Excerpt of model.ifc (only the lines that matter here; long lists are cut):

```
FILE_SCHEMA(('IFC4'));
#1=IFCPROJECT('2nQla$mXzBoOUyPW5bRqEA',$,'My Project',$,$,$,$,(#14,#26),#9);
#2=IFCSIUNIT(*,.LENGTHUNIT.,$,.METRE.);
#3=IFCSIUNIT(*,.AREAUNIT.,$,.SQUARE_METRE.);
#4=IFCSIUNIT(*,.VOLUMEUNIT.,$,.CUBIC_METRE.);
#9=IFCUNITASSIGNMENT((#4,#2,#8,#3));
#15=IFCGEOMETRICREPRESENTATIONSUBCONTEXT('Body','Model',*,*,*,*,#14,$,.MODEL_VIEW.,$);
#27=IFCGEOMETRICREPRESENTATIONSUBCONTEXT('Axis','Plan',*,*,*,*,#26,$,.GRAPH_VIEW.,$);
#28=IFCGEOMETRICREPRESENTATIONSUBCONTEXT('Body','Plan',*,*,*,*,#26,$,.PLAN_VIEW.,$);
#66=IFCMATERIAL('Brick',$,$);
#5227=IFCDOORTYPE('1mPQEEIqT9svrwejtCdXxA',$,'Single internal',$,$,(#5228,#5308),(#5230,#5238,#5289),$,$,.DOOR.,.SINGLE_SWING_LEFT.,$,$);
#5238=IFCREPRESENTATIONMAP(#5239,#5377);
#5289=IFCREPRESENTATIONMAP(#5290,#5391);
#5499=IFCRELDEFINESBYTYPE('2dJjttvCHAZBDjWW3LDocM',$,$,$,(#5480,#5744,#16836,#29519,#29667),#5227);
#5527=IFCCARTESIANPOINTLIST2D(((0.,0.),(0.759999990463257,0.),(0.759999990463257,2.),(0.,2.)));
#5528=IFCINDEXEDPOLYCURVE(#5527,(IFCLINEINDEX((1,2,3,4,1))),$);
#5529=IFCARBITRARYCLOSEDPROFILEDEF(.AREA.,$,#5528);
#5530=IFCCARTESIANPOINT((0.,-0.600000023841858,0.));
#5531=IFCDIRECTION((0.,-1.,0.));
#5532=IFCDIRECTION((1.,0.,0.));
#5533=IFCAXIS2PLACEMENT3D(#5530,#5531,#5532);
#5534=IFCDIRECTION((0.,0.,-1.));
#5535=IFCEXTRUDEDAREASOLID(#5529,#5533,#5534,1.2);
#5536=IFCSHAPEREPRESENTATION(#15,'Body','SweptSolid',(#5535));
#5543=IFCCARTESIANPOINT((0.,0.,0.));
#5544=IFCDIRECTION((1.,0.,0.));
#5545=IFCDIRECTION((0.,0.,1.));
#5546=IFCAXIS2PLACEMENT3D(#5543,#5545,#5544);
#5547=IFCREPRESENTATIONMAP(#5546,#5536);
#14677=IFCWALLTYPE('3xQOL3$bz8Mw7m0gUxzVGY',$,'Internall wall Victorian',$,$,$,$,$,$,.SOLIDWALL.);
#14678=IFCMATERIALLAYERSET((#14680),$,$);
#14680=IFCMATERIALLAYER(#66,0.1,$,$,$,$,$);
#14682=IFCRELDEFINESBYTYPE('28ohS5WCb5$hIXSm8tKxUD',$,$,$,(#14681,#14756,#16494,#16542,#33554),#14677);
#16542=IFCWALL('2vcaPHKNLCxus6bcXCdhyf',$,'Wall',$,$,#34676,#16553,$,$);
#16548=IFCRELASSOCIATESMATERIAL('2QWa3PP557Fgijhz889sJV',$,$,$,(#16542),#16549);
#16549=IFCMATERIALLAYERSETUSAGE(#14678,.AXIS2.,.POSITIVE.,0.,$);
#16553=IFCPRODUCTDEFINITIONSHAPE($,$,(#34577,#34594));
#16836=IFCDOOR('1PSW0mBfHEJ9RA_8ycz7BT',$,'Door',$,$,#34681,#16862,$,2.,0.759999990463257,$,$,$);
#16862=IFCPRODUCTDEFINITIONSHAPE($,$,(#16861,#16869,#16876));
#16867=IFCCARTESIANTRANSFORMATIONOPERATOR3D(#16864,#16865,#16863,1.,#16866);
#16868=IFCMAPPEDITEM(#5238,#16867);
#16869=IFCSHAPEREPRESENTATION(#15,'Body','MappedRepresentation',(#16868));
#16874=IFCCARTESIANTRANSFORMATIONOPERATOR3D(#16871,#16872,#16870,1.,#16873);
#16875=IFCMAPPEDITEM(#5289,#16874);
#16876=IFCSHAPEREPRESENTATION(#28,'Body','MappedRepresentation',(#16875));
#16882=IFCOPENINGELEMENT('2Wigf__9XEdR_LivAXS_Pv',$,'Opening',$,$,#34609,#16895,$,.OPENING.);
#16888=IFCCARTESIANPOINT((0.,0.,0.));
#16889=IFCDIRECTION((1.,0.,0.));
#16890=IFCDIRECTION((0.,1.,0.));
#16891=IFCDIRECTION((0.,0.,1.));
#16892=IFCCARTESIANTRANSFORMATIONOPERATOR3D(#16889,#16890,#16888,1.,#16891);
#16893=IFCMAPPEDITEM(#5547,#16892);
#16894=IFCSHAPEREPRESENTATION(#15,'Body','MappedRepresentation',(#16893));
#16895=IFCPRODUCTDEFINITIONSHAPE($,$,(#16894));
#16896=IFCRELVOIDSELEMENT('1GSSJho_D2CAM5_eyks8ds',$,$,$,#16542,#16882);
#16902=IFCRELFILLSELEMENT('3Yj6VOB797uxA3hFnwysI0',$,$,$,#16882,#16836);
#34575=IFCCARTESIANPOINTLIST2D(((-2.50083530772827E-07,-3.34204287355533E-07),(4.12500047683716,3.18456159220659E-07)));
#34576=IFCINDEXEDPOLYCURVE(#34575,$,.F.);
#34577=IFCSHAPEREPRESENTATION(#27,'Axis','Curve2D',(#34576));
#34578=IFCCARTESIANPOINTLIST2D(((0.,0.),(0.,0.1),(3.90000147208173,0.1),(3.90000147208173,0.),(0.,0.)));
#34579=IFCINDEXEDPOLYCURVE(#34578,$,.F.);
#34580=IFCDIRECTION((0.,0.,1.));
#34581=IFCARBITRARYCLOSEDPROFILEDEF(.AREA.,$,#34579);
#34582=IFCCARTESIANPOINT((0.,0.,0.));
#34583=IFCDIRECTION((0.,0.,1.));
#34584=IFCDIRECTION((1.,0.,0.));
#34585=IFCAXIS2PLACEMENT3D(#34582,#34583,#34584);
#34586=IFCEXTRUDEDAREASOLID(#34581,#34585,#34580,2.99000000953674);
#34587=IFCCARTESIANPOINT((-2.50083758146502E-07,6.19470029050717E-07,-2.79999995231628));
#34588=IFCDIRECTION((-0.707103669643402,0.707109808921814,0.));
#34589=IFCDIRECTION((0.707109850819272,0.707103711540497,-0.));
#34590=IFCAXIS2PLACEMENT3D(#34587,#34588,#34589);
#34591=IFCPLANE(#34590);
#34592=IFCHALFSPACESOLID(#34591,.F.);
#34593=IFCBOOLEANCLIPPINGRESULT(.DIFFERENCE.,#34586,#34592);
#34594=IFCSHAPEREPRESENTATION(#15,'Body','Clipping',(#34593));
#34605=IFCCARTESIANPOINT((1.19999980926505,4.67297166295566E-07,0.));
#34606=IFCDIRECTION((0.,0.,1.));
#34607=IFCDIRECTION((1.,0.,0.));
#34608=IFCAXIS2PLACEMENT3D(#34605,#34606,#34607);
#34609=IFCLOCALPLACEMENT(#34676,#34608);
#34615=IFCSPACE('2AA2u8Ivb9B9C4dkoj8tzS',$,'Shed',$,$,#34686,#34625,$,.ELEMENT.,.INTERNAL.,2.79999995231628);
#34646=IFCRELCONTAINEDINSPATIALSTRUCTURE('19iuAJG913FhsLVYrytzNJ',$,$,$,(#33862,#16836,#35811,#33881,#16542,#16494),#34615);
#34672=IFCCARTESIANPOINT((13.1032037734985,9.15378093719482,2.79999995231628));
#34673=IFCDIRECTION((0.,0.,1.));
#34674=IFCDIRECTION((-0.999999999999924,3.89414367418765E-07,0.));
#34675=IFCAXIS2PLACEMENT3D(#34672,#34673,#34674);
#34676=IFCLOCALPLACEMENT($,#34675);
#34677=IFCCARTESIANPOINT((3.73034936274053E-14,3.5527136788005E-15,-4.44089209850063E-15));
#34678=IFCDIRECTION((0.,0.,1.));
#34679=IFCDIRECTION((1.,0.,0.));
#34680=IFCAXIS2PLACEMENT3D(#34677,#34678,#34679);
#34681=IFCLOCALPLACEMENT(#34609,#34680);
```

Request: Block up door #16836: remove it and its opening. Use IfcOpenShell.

```python
import ifcopenshell
import ifcopenshell.api.feature
import ifcopenshell.api.root
import ifcopenshell.geom
import ifcopenshell.util.shape

model = ifcopenshell.open("model.ifc")
settings = ifcopenshell.geom.settings()


def volume(element):
    """Net volume in cubic metres, openings subtracted."""
    shape = ifcopenshell.geom.create_shape(settings, element)
    return ifcopenshell.util.shape.get_volume(shape.geometry)


door = model.by_guid("1PSW0mBfHEJ9RA_8ycz7BT")
opening = door.FillsVoids[0].RelatingOpeningElement
wall = opening.VoidsElements[0].RelatingBuildingElement
before = volume(wall)

ifcopenshell.api.root.remove_product(model, product=door)
ifcopenshell.api.feature.remove_feature(model, feature=opening)

after = volume(wall)

print(f"wall volume {before:.3f} -> {after:.3f} m3")

model.write("model-out.ifc")
```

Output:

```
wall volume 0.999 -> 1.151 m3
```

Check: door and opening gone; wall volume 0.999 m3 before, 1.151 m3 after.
